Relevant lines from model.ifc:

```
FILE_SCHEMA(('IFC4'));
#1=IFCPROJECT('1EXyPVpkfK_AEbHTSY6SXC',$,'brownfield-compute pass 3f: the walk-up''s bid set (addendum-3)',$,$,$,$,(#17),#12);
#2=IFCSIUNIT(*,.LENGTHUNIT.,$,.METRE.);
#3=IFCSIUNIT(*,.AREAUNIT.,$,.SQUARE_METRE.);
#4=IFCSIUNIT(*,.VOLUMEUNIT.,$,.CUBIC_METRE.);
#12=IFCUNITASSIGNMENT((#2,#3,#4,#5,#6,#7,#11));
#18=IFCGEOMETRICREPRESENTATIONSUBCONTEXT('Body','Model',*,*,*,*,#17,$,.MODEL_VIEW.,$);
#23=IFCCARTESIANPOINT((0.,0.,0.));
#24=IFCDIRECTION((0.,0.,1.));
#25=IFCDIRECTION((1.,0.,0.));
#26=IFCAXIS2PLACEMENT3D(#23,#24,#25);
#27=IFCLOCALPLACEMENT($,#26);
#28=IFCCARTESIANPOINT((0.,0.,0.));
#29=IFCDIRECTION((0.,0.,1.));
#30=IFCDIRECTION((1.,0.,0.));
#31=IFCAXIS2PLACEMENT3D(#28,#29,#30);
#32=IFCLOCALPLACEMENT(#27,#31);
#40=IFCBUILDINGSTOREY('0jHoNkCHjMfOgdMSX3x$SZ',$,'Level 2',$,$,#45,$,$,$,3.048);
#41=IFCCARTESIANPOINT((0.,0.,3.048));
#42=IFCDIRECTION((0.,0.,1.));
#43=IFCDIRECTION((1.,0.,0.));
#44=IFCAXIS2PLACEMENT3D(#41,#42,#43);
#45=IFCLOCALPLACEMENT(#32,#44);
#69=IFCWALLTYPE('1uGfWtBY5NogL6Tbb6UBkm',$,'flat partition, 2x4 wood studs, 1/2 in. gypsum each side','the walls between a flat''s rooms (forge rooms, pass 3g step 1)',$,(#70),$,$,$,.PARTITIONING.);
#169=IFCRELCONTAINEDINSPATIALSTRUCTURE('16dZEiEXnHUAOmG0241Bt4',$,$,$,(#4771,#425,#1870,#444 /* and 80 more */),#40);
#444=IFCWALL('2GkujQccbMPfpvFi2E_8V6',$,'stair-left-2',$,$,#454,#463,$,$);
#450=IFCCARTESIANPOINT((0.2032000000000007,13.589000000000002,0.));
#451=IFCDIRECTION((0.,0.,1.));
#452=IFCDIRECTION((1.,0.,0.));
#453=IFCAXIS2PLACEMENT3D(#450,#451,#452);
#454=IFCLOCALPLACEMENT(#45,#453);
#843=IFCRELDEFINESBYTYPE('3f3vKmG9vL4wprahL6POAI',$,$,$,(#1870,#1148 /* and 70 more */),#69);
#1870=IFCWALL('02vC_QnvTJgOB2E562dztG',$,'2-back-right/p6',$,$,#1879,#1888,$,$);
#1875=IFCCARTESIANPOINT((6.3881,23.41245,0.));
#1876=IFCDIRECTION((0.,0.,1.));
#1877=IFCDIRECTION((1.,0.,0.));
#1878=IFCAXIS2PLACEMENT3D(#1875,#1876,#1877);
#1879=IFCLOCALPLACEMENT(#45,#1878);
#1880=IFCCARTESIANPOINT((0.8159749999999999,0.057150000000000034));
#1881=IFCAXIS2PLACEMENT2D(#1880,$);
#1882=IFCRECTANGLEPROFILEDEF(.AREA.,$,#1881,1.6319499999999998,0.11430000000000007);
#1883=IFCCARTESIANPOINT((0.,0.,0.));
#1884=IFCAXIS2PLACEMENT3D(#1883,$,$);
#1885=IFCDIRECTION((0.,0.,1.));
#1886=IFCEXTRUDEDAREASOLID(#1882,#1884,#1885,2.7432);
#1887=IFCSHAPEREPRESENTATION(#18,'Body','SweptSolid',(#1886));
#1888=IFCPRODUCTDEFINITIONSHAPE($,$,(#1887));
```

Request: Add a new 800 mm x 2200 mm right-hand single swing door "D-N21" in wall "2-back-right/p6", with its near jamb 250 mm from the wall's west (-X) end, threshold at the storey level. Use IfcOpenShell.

```python
import numpy as np
import ifcopenshell
import ifcopenshell.api.feature
import ifcopenshell.api.geometry
import ifcopenshell.api.root
import ifcopenshell.api.spatial
import ifcopenshell.geom
import ifcopenshell.util.element
import ifcopenshell.util.placement
import ifcopenshell.util.representation
import ifcopenshell.util.shape
import ifcopenshell.util.unit

model = ifcopenshell.open("model.ifc")
unit_scale = ifcopenshell.util.unit.calculate_unit_scale(model)
settings = ifcopenshell.geom.settings()


def volume(element):
    """Net volume in cubic metres, openings subtracted."""
    shape = ifcopenshell.geom.create_shape(settings, element)
    return ifcopenshell.util.shape.get_volume(shape.geometry)


wall = model.by_guid("02vC_QnvTJgOB2E562dztG")
storey = ifcopenshell.util.element.get_container(wall, ifc_class="IfcBuildingStorey")
context = ifcopenshell.util.representation.get_context(model, "Model", "Body", "MODEL_VIEW")
before = volume(wall)

width, height, from_end, sill = 0.8, 2.2, 0.25, 0.0  # metres

# The wall runs along its own X axis, and the end named is its -X end.
wall_shape = ifcopenshell.geom.create_shape(settings, wall)
x, y, z = ifcopenshell.util.shape.get_vertices(wall_shape.geometry).T
start = x.min() + from_end
face, thickness = float(y.min()), float(y.max() - y.min())
wall_matrix = ifcopenshell.util.placement.get_local_placement(wall.ObjectPlacement)
level = ifcopenshell.util.placement.get_local_placement(storey.ObjectPlacement)[2, 3]


def in_wall(x, y):
    """Placement at x, y metres in the wall's axes, at sill height."""
    matrix = wall_matrix.copy()
    matrix[:, 3] = wall_matrix @ np.array([x / unit_scale, y / unit_scale, 0.0, 1.0])
    matrix[2, 3] = level + sill / unit_scale
    return matrix


# Opening: a box that overshoots both wall faces by 50 mm.
opening = ifcopenshell.api.root.create_entity(model, ifc_class="IfcOpeningElement", predefined_type="OPENING")
box = ifcopenshell.api.geometry.add_wall_representation(
    model, context=context, length=width, height=height, thickness=thickness + 0.1
)
ifcopenshell.api.geometry.assign_representation(model, product=opening, representation=box)
ifcopenshell.api.geometry.edit_object_placement(model, product=opening, matrix=in_wall(start, face - 0.05), is_si=False)
ifcopenshell.api.feature.add_feature(model, feature=opening, element=wall)

door = ifcopenshell.api.root.create_entity(model, ifc_class="IfcDoor", name="D-N21", predefined_type="DOOR")
door.OverallWidth, door.OverallHeight = width / unit_scale, height / unit_scale
door.OperationType = "SINGLE_SWING_RIGHT"
body = ifcopenshell.api.geometry.add_door_representation(
    model,
    context=context,
    overall_width=door.OverallWidth,
    overall_height=door.OverallHeight,
    operation_type="SINGLE_SWING_RIGHT",
    lining_properties={"LiningDepth": thickness / unit_scale, "ThresholdDepth": thickness / unit_scale},
)
ifcopenshell.api.geometry.assign_representation(model, product=door, representation=body)
ifcopenshell.api.spatial.assign_container(model, products=[door], relating_structure=storey)
ifcopenshell.api.feature.add_filling(model, opening=opening, element=door)

# The lining spans the wall, so the door starts at the wall face.
ifcopenshell.api.geometry.edit_object_placement(model, product=door, matrix=in_wall(start, face), is_si=False)

after = volume(wall)

print(f"wall volume {before:.3f} -> {after:.3f} m3")

model.write("model_rev.ifc")
```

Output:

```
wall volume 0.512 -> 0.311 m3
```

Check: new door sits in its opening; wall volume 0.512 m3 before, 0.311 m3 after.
